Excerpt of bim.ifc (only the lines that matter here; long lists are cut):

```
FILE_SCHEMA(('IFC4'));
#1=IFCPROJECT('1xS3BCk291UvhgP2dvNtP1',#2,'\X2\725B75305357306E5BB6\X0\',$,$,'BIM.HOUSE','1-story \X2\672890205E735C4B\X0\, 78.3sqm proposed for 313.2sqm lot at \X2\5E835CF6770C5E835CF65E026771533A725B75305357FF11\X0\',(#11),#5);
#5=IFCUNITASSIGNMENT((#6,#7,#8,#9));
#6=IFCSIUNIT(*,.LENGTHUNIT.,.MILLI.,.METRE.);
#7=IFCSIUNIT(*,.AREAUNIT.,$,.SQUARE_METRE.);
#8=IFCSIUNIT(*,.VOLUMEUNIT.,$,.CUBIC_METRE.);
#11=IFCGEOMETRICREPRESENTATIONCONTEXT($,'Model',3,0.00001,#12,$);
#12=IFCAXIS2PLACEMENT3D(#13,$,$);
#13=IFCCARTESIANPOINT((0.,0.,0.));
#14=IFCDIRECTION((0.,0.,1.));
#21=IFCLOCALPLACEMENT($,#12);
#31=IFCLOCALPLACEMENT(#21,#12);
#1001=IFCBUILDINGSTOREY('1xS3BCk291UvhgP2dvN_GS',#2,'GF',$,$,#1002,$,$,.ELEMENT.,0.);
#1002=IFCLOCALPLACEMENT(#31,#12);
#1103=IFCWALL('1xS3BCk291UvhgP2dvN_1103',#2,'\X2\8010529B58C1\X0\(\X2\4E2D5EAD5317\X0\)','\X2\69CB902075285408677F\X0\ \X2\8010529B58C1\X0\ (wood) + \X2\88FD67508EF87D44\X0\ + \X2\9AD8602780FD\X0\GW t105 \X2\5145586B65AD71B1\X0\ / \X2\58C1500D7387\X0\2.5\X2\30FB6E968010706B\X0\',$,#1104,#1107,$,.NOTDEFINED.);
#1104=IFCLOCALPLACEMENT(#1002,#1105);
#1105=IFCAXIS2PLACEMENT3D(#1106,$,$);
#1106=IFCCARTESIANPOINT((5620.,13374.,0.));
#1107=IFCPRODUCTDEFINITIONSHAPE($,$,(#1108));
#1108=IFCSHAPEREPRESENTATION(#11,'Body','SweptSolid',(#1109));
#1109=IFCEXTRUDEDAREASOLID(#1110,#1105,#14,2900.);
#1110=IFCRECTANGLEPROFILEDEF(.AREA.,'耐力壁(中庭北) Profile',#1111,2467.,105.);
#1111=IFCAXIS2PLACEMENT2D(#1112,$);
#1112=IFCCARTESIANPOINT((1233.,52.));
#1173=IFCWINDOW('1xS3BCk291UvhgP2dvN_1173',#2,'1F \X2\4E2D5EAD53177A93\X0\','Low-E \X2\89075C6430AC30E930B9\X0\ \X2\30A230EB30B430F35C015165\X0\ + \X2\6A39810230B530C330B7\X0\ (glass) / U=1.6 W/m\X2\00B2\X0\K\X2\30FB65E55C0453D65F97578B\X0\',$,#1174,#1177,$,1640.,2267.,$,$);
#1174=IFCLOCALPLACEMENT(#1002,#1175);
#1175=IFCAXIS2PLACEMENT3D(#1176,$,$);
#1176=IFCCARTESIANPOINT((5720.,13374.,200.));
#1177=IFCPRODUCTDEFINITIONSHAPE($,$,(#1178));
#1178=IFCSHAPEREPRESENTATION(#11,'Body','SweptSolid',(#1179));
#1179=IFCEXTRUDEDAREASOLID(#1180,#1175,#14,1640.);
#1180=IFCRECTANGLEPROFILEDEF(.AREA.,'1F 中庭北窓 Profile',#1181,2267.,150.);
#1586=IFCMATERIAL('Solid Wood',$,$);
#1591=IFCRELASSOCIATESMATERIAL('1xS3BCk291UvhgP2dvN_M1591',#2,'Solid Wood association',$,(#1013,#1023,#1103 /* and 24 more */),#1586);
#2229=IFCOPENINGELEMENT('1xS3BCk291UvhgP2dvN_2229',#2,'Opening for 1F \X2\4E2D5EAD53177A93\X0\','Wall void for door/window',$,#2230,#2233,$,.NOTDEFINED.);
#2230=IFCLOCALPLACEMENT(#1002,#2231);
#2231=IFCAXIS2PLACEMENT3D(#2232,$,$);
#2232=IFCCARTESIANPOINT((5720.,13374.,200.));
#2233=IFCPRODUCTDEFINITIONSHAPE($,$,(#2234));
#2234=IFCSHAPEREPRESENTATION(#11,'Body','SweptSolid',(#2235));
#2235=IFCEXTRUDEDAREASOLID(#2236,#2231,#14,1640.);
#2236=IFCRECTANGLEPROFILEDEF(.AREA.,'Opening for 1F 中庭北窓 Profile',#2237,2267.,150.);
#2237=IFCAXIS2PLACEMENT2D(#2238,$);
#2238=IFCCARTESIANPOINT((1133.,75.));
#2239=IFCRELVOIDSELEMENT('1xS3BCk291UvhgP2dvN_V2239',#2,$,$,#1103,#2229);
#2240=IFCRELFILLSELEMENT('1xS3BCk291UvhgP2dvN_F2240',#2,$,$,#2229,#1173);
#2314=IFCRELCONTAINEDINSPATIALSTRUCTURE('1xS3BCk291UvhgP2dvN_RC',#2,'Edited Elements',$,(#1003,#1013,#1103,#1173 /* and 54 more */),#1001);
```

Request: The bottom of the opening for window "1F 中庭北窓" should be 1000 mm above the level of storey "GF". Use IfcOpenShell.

```python
import numpy as np
import ifcopenshell
import ifcopenshell.api.geometry
import ifcopenshell.geom
import ifcopenshell.util.element
import ifcopenshell.util.placement
import ifcopenshell.util.shape
import ifcopenshell.util.unit

model = ifcopenshell.open("bim.ifc")
unit_scale = ifcopenshell.util.unit.calculate_unit_scale(model)

window = model.by_id(1173)
opening = window.FillsVoids[0].RelatingOpeningElement
storey = ifcopenshell.util.element.get_container(window, ifc_class="IfcBuildingStorey")
level = ifcopenshell.util.placement.get_local_placement(storey.ObjectPlacement)[2, 3]

# The opening's origin need not be at the sill, so measure its lowest point.
shape = ifcopenshell.geom.create_shape(ifcopenshell.geom.settings(), opening)
bottom = ifcopenshell.util.shape.get_shape_bottom_elevation(shape, shape.geometry) / unit_scale
dz = level + 1000.0 - bottom

shift = np.array([0.0, 0.0, dz])
# The window is not placed relative to its opening, so move both.
for product in (opening, window):
    matrix = ifcopenshell.util.placement.get_local_placement(product.ObjectPlacement)
    matrix[:3, 3] += shift
    ifcopenshell.api.geometry.edit_object_placement(model, product=product, matrix=matrix, is_si=False)

print(f"moved by {dz * unit_scale:+.3f} m")

model.write("bim_rev.ifc")
```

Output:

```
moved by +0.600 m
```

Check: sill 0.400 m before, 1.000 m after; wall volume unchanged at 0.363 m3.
